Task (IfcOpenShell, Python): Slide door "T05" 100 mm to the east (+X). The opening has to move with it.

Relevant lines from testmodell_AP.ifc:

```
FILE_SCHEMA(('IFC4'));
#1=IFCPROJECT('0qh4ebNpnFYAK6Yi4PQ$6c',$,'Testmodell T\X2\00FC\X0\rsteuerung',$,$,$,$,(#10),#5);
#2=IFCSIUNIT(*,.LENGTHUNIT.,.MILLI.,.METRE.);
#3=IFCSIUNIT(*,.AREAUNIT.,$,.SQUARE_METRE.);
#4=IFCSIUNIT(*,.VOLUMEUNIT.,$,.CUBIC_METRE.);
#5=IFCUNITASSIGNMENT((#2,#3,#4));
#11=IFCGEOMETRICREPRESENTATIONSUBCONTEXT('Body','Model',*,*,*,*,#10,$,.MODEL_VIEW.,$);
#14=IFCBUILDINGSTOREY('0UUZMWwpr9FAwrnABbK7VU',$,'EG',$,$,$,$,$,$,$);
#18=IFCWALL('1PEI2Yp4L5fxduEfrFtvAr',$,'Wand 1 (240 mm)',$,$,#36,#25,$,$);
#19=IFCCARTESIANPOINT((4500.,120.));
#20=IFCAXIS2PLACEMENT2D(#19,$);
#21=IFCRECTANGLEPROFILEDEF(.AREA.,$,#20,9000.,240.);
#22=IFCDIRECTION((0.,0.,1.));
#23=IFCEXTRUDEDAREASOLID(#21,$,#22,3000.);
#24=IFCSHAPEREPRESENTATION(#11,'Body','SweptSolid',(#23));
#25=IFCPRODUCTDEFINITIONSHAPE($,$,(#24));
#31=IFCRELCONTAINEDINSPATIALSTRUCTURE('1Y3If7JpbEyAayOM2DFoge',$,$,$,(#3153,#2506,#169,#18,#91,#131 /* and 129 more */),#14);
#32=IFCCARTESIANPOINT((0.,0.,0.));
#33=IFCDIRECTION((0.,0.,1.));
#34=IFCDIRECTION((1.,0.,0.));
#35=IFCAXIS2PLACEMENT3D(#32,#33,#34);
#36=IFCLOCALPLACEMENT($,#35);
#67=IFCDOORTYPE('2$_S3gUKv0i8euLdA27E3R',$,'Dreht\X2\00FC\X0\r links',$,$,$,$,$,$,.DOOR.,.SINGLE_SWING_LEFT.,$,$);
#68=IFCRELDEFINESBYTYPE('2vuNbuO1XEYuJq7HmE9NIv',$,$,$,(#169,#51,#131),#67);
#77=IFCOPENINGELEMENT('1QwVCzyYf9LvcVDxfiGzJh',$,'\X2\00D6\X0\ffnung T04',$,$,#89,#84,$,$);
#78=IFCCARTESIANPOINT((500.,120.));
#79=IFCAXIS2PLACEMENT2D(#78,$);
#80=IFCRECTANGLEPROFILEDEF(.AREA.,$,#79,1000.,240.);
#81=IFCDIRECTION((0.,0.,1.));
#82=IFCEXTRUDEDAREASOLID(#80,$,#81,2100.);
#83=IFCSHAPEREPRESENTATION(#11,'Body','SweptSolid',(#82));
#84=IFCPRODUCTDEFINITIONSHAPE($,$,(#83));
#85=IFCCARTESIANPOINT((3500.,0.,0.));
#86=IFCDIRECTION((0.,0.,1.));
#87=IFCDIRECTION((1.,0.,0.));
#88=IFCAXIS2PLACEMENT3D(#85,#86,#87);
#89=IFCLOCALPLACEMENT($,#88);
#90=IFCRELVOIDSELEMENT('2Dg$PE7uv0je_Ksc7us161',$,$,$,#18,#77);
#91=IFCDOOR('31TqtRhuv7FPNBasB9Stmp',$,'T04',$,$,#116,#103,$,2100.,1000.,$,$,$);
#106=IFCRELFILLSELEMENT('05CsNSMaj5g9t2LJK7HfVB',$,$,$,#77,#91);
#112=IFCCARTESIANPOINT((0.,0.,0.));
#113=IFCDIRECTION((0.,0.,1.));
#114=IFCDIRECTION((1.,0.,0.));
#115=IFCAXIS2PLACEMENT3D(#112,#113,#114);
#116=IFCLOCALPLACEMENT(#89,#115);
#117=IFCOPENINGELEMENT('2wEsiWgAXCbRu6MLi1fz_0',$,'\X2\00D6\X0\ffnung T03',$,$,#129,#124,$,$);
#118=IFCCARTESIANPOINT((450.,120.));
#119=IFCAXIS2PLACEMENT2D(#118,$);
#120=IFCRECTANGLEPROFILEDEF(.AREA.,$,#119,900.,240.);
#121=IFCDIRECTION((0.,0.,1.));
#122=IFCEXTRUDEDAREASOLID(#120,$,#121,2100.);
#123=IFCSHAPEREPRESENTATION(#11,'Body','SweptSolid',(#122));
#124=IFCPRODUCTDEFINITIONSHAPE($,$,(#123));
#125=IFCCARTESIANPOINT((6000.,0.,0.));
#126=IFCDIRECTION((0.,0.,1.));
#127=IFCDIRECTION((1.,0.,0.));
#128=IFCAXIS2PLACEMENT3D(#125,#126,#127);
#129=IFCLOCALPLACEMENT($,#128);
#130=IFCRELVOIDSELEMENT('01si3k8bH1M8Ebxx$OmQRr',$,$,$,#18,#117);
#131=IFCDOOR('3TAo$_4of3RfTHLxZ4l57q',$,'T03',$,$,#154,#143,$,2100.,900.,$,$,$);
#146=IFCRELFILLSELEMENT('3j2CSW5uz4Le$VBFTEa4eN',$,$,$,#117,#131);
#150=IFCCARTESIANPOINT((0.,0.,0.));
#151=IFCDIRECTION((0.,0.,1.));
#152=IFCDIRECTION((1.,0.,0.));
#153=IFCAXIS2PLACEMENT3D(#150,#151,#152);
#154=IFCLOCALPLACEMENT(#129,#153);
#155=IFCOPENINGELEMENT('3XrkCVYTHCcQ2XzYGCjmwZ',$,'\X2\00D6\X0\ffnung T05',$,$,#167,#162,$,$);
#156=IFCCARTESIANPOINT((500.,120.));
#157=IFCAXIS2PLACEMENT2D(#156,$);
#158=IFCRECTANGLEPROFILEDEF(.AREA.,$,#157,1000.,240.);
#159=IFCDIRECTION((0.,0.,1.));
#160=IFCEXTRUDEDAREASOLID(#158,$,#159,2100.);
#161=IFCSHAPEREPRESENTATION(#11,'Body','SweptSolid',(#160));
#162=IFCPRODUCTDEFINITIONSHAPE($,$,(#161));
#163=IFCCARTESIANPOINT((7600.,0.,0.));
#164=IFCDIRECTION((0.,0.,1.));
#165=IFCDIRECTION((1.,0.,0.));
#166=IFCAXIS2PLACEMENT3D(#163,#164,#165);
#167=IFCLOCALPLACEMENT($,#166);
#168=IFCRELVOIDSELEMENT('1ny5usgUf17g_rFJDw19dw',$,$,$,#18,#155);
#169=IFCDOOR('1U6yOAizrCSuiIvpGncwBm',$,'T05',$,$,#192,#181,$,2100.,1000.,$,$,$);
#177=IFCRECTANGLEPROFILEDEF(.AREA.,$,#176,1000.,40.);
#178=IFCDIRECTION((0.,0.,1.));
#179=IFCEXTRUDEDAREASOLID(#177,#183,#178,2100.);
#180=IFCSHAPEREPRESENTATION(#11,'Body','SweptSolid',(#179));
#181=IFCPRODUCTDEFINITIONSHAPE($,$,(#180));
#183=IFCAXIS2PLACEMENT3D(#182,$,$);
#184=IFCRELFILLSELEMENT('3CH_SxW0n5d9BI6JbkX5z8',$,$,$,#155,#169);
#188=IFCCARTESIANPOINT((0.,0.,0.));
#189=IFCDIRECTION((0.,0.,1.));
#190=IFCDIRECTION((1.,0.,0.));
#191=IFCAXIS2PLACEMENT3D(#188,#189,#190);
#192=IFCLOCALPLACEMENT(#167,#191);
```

```python
import ifcopenshell
import ifcopenshell.api.geometry
import ifcopenshell.util.placement
import ifcopenshell.util.unit

model = ifcopenshell.open("testmodell_AP.ifc")
unit_scale = ifcopenshell.util.unit.calculate_unit_scale(model)

door = model.by_id(169)
opening = door.FillsVoids[0].RelatingOpeningElement
wall = opening.VoidsElements[0].RelatingBuildingElement

wall_matrix = ifcopenshell.util.placement.get_local_placement(wall.ObjectPlacement)
shift = wall_matrix[:3, 0] * 0.1 / unit_scale
before = ifcopenshell.util.placement.get_local_placement(door.ObjectPlacement)[:3, 3].copy()

# The door is placed relative to its opening, so it follows when the opening moves.
matrix = ifcopenshell.util.placement.get_local_placement(opening.ObjectPlacement)
matrix[:3, 3] += shift
ifcopenshell.api.geometry.edit_object_placement(
    model, product=opening, matrix=matrix, is_si=False, should_transform_children=True
)

after = ifcopenshell.util.placement.get_local_placement(door.ObjectPlacement)[:3, 3]
print("door moved by", (after - before).round(3) + 0.0)

model.write("testmodell_AP_v2.ifc")
```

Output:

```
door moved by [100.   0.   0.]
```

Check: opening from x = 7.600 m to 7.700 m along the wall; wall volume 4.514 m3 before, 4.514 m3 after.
